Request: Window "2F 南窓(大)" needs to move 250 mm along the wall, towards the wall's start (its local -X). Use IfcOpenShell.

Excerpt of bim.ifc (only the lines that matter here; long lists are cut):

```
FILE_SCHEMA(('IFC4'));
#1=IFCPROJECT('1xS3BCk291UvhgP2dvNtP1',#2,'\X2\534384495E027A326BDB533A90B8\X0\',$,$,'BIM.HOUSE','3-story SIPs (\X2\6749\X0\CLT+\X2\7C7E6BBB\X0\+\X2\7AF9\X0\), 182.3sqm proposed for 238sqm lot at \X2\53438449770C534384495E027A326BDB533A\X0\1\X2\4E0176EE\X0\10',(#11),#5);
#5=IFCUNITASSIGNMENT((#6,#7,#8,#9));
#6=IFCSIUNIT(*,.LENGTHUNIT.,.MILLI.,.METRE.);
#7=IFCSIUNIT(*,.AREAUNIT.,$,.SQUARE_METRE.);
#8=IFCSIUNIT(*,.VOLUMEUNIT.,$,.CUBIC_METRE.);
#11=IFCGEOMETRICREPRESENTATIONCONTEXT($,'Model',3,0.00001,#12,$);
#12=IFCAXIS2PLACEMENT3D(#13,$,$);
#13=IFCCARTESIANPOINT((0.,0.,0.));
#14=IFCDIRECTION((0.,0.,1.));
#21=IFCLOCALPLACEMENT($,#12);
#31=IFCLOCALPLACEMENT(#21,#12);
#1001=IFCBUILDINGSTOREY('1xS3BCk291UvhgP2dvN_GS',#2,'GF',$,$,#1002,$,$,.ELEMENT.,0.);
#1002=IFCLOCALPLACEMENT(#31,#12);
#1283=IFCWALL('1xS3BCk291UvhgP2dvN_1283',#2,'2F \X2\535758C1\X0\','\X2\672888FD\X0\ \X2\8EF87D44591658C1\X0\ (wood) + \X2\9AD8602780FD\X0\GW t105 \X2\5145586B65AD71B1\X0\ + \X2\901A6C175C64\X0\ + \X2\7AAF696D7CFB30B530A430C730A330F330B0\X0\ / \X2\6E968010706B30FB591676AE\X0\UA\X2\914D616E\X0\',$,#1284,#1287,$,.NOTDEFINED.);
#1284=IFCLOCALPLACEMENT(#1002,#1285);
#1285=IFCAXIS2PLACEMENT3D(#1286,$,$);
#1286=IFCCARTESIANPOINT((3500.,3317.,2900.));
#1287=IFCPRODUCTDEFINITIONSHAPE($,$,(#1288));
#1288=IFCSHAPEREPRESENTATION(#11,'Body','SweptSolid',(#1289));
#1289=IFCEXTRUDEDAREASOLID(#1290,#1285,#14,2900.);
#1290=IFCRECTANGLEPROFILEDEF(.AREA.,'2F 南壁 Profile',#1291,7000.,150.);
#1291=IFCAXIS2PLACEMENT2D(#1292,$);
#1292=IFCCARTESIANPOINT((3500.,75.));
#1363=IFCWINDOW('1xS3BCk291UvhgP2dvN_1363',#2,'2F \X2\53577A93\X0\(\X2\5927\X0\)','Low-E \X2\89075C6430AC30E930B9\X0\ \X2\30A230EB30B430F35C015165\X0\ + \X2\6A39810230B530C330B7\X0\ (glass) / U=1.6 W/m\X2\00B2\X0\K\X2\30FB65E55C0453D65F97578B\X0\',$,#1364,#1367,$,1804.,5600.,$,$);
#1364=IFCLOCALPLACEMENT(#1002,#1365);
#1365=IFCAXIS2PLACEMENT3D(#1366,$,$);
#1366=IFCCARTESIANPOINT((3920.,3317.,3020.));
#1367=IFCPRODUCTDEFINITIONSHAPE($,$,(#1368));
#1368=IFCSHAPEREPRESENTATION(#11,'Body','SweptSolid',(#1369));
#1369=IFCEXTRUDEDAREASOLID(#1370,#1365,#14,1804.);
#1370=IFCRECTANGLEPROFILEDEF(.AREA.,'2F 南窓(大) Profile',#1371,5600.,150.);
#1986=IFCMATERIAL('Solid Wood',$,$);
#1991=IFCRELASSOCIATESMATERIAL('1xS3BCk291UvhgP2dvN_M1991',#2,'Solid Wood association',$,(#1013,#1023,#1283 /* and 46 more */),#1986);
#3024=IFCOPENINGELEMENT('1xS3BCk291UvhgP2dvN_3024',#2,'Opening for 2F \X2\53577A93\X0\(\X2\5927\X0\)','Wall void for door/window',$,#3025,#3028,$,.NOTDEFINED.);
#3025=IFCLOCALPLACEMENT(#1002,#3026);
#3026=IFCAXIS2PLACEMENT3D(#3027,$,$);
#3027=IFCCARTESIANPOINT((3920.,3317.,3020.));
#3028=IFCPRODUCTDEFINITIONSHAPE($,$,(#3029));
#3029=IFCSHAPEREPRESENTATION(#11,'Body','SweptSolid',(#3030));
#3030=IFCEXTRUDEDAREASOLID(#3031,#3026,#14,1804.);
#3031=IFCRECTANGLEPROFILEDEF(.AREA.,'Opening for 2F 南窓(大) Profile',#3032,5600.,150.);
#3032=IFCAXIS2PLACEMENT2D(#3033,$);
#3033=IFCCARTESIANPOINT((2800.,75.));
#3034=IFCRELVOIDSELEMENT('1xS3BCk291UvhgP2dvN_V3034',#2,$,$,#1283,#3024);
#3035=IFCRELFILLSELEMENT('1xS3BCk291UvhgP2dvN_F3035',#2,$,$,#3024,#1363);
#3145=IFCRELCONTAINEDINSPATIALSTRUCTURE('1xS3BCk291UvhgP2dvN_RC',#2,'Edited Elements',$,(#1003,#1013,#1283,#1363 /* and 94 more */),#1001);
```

```python
import ifcopenshell
import ifcopenshell.api.geometry
import ifcopenshell.util.placement
import ifcopenshell.util.unit

model = ifcopenshell.open("bim.ifc")
unit_scale = ifcopenshell.util.unit.calculate_unit_scale(model)

window = model.by_id(1363)
opening = window.FillsVoids[0].RelatingOpeningElement
wall = opening.VoidsElements[0].RelatingBuildingElement

wall_matrix = ifcopenshell.util.placement.get_local_placement(wall.ObjectPlacement)
shift = wall_matrix[:3, 0] * -0.25 / unit_scale
before = ifcopenshell.util.placement.get_local_placement(window.ObjectPlacement)[:3, 3].copy()

# The window is not placed relative to its opening, so move both.
for product in (opening, window):
    matrix = ifcopenshell.util.placement.get_local_placement(product.ObjectPlacement)
    matrix[:3, 3] += shift
    ifcopenshell.api.geometry.edit_object_placement(model, product=product, matrix=matrix, is_si=False)

after = ifcopenshell.util.placement.get_local_placement(window.ObjectPlacement)[:3, 3]
print("window moved by", (after - before).round(3) + 0.0)

model.write("bim_edited.ifc")
```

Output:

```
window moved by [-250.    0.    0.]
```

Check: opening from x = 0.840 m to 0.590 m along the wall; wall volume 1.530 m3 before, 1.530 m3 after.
